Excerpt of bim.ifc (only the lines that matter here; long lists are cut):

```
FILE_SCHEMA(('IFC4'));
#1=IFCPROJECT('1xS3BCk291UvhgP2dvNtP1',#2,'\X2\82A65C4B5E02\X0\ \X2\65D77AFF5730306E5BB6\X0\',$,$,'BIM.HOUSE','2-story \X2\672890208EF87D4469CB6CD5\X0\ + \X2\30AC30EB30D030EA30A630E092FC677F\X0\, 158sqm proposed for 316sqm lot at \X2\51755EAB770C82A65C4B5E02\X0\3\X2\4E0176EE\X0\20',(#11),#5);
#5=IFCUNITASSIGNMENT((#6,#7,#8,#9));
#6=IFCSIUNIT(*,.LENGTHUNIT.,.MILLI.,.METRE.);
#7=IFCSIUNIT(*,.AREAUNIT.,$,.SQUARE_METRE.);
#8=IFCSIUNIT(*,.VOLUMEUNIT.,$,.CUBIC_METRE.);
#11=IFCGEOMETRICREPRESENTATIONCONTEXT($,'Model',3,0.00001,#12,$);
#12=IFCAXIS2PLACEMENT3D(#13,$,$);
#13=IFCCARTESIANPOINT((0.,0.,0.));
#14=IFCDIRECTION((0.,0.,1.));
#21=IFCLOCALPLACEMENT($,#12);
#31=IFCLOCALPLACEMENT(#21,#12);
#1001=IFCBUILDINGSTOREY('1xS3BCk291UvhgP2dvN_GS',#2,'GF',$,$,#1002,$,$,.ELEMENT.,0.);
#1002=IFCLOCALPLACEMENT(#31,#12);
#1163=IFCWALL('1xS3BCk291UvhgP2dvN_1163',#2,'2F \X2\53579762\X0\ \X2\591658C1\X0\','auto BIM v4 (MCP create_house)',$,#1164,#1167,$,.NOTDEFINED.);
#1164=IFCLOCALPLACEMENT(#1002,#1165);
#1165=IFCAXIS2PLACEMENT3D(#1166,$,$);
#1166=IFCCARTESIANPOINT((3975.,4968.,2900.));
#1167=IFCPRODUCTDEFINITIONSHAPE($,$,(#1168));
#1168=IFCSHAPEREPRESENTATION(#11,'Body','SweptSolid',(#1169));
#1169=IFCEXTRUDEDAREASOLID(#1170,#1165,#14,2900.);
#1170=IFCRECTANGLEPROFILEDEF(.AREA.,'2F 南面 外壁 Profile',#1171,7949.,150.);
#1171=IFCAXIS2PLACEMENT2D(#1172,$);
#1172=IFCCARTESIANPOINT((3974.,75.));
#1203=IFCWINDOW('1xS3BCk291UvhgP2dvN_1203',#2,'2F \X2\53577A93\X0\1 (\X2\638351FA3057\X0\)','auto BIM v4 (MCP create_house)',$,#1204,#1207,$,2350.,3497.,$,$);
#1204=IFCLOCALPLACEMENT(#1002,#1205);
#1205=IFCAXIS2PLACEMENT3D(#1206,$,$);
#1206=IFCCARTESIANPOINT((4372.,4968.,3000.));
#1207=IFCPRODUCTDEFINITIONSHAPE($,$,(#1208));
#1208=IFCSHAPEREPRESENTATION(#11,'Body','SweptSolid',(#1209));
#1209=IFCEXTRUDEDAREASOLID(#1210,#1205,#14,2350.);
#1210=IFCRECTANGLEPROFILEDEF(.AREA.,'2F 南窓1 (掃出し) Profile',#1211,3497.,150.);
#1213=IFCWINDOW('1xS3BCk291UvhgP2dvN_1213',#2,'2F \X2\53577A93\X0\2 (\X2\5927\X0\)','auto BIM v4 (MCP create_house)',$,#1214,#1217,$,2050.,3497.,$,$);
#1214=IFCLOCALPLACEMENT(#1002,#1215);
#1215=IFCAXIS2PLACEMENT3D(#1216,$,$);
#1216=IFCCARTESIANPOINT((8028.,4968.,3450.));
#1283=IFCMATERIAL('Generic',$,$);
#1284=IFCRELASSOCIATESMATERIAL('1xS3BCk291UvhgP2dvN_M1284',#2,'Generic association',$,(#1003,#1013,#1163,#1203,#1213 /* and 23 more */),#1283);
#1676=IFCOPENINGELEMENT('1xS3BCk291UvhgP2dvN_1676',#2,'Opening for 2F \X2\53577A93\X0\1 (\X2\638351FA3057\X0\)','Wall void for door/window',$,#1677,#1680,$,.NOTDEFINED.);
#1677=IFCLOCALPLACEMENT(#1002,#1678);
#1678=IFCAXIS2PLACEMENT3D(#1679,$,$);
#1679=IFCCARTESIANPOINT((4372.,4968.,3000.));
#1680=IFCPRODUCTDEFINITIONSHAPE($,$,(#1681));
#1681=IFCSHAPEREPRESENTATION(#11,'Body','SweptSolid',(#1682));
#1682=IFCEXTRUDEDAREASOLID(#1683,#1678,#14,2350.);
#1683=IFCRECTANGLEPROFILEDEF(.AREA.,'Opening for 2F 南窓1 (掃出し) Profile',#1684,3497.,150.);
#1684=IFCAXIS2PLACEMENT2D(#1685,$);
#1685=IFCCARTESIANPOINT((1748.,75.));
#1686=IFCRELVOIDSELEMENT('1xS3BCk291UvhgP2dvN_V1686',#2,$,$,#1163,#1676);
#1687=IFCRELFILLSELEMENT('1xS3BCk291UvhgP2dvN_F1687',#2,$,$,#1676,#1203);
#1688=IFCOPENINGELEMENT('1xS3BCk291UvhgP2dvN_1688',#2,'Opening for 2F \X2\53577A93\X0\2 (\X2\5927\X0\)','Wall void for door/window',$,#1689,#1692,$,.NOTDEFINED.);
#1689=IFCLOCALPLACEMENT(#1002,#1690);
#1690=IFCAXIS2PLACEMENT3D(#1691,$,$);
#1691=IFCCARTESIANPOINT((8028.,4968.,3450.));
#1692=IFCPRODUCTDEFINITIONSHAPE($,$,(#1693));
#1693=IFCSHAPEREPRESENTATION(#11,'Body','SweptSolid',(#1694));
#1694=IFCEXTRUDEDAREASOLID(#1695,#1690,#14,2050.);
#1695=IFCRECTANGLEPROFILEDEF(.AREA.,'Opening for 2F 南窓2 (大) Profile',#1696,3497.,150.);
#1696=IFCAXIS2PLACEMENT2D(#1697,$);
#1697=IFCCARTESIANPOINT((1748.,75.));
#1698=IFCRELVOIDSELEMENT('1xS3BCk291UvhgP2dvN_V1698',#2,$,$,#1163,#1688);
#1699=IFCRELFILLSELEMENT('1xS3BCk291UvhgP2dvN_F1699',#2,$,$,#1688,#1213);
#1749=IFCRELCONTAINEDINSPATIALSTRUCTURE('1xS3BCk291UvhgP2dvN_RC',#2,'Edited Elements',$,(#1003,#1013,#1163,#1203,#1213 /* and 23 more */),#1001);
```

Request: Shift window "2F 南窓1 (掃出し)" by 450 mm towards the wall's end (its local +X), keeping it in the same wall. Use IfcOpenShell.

```python
import ifcopenshell
import ifcopenshell.api.geometry
import ifcopenshell.util.placement
import ifcopenshell.util.unit

model = ifcopenshell.open("bim.ifc")
unit_scale = ifcopenshell.util.unit.calculate_unit_scale(model)

window = model.by_guid("1xS3BCk291UvhgP2dvN_1203")
opening = window.FillsVoids[0].RelatingOpeningElement
wall = opening.VoidsElements[0].RelatingBuildingElement

wall_matrix = ifcopenshell.util.placement.get_local_placement(wall.ObjectPlacement)
shift = wall_matrix[:3, 0] * 0.45 / unit_scale
before = ifcopenshell.util.placement.get_local_placement(window.ObjectPlacement)[:3, 3].copy()

# The window is not placed relative to its opening, so move both.
for product in (opening, window):
    matrix = ifcopenshell.util.placement.get_local_placement(product.ObjectPlacement)
    matrix[:3, 3] += shift
    ifcopenshell.api.geometry.edit_object_placement(model, product=product, matrix=matrix, is_si=False)

after = ifcopenshell.util.placement.get_local_placement(window.ObjectPlacement)[:3, 3]
print("window moved by", (after - before).round(3) + 0.0)

model.write("bim_edited.ifc")
```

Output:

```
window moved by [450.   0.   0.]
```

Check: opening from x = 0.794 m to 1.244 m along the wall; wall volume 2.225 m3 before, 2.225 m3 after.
